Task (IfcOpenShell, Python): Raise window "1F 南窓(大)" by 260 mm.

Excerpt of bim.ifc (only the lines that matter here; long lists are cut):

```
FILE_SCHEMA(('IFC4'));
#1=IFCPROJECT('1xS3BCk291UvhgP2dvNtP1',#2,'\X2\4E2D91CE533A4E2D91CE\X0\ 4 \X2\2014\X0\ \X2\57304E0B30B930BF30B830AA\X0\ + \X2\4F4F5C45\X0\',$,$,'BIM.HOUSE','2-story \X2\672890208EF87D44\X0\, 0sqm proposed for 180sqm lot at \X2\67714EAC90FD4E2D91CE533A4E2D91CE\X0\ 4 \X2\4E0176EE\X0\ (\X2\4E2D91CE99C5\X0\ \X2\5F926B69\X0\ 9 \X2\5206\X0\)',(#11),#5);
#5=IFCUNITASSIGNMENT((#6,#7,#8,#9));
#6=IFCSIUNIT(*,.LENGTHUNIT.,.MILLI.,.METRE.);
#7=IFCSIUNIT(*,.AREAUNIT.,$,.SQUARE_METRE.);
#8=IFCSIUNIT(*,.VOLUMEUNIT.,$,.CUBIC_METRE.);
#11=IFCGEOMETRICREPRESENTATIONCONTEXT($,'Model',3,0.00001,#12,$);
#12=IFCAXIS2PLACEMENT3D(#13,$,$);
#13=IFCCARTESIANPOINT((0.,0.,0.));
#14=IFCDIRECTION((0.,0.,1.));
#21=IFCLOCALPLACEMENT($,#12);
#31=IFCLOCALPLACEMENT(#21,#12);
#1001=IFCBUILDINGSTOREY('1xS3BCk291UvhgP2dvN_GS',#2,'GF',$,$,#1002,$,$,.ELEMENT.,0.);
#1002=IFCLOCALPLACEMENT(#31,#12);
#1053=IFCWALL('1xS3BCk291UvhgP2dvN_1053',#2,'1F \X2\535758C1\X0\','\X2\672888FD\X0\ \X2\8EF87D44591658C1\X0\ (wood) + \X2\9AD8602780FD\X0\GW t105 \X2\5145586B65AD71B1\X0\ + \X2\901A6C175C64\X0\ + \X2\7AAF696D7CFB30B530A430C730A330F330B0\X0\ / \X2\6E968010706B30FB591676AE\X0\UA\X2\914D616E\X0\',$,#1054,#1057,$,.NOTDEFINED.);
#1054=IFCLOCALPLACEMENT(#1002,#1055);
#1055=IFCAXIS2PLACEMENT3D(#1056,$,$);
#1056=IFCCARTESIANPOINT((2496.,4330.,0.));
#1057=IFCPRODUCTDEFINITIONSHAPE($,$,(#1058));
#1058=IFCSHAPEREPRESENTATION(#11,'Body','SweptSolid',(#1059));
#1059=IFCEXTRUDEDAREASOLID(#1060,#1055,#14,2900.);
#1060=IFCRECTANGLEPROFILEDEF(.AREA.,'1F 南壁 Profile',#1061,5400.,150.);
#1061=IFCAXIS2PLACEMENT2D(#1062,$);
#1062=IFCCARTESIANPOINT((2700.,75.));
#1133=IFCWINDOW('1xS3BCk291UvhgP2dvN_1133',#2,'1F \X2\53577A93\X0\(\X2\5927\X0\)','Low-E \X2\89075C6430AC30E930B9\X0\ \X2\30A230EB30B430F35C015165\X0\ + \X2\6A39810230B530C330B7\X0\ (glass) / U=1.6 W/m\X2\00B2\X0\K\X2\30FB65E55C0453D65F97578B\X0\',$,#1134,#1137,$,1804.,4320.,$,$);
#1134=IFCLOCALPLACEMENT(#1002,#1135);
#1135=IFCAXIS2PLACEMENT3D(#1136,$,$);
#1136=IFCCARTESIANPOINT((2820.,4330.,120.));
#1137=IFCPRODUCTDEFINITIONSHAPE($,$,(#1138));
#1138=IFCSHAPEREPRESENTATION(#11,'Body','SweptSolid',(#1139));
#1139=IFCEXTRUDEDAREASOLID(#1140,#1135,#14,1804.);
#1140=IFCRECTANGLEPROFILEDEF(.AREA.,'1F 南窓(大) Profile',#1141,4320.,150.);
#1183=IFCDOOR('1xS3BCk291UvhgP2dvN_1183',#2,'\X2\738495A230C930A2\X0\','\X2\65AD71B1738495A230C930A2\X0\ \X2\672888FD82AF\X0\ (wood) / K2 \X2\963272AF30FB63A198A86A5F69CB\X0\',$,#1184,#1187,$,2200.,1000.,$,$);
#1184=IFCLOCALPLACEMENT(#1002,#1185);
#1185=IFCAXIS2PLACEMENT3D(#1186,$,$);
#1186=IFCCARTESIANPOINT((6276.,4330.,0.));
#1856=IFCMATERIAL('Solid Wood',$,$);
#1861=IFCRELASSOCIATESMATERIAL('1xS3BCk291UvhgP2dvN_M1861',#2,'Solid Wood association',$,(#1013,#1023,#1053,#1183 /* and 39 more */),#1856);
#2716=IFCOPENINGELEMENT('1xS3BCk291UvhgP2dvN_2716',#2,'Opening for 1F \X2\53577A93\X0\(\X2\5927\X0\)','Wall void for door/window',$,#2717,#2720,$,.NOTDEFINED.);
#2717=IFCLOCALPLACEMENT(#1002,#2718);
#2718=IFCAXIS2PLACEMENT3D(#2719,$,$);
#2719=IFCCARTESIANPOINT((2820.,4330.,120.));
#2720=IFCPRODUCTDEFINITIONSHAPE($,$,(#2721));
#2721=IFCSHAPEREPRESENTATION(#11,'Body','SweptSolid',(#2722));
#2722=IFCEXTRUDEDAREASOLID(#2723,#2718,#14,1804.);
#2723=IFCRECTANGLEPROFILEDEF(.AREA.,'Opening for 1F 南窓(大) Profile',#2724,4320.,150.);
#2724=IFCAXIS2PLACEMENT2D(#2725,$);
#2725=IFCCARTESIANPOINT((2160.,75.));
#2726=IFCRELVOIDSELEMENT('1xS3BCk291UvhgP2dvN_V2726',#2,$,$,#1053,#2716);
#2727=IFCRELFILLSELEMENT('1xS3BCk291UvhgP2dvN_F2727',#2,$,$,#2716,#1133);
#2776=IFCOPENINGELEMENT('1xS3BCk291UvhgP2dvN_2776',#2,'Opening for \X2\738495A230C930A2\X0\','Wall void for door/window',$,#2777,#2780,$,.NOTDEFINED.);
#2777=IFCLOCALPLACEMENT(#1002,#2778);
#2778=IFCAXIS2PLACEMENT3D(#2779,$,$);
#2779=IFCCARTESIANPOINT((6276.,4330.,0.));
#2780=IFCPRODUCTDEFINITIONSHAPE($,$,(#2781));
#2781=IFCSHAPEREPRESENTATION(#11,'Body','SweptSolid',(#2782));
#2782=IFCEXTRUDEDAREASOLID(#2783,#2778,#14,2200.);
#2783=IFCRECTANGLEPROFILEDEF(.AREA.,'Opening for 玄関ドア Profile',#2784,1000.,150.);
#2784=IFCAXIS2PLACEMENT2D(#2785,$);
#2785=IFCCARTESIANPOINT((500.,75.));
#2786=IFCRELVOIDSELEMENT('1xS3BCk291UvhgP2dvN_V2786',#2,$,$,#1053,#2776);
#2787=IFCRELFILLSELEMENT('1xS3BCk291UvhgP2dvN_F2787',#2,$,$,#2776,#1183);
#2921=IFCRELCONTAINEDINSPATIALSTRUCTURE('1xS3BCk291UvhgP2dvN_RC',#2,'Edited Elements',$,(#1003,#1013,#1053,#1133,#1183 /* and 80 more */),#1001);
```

```python
import numpy as np
import ifcopenshell
import ifcopenshell.api.geometry
import ifcopenshell.util.placement
import ifcopenshell.util.unit

model = ifcopenshell.open("bim.ifc")
unit_scale = ifcopenshell.util.unit.calculate_unit_scale(model)

window = model.by_guid("1xS3BCk291UvhgP2dvN_1133")
opening = window.FillsVoids[0].RelatingOpeningElement
dz = 260.0

shift = np.array([0.0, 0.0, dz])
# The window is not placed relative to its opening, so move both.
for product in (opening, window):
    matrix = ifcopenshell.util.placement.get_local_placement(product.ObjectPlacement)
    matrix[:3, 3] += shift
    ifcopenshell.api.geometry.edit_object_placement(model, product=product, matrix=matrix, is_si=False)

print(f"moved by {dz * unit_scale:+.3f} m")

model.write("bim_rev.ifc")
```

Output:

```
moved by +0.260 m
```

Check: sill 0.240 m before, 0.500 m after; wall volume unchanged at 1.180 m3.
